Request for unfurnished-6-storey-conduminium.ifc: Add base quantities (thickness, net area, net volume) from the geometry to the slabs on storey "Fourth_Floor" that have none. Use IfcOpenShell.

First a look at what the model holds.

```python
import ifcopenshell
import ifcopenshell.util.element
import ifcopenshell.util.unit

model = ifcopenshell.open("unfurnished-6-storey-conduminium.ifc")
print(model.schema)
for unit_type in ("LENGTHUNIT", "AREAUNIT", "VOLUMEUNIT"):
    print(unit_type, ifcopenshell.util.unit.calculate_unit_scale(model, unit_type))
storey = next(s for s in model.by_type("IfcBuildingStorey") if s.Name == "Fourth_Floor")
slabs = [e for e in ifcopenshell.util.element.get_decomposition(storey) if e.is_a("IfcSlab")]
for e in sorted(slabs, key=lambda e: e.id()):
    print(e.id(), e.is_a(), e.Name, list(ifcopenshell.util.element.get_psets(e, qtos_only=True)), sep=" | ")
```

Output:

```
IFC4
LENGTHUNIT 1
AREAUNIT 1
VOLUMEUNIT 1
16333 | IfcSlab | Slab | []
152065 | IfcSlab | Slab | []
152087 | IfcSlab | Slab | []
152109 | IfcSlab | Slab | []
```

```python
import ifcopenshell
import ifcopenshell.api.pset
import ifcopenshell.geom
import ifcopenshell.util.element
import ifcopenshell.util.shape
import ifcopenshell.util.unit

model = ifcopenshell.open("unfurnished-6-storey-conduminium.ifc")
unit_scale = ifcopenshell.util.unit.calculate_unit_scale(model)
area_scale = ifcopenshell.util.unit.calculate_unit_scale(model, "AREAUNIT")
volume_scale = ifcopenshell.util.unit.calculate_unit_scale(model, "VOLUMEUNIT")
settings = ifcopenshell.geom.settings()

storey = next(s for s in model.by_type("IfcBuildingStorey") if s.Name == "Fourth_Floor")
slabs = [e for e in ifcopenshell.util.element.get_decomposition(storey) if e.is_a("IfcSlab")]

for e in sorted(slabs, key=lambda e: e.id()):
    if ifcopenshell.util.element.get_psets(e, qtos_only=True, should_inherit=False):
        continue
    # Geometry comes back in metres, in the element's own axes.
    shape = ifcopenshell.geom.create_shape(settings, e)
    values = {
        "Width": ifcopenshell.util.shape.get_z(shape.geometry) / unit_scale,
        "NetArea": ifcopenshell.util.shape.get_footprint_area(shape.geometry) / area_scale,
        "NetVolume": ifcopenshell.util.shape.get_volume(shape.geometry) / volume_scale,
    }
    qto = ifcopenshell.api.pset.add_qto(model, product=e, name="Qto_SlabBaseQuantities")
    ifcopenshell.api.pset.edit_qto(model, qto=qto, properties=values)
    print(e.id(), {k: round(v, 3) for k, v in values.items()})

model.write("unfurnished-6-storey-conduminium_v2.ifc")
```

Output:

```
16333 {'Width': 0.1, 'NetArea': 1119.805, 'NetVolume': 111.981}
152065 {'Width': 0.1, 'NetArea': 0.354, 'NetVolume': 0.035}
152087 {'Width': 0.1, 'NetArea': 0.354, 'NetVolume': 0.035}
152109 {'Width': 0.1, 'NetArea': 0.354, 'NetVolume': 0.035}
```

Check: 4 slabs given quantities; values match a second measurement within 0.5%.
